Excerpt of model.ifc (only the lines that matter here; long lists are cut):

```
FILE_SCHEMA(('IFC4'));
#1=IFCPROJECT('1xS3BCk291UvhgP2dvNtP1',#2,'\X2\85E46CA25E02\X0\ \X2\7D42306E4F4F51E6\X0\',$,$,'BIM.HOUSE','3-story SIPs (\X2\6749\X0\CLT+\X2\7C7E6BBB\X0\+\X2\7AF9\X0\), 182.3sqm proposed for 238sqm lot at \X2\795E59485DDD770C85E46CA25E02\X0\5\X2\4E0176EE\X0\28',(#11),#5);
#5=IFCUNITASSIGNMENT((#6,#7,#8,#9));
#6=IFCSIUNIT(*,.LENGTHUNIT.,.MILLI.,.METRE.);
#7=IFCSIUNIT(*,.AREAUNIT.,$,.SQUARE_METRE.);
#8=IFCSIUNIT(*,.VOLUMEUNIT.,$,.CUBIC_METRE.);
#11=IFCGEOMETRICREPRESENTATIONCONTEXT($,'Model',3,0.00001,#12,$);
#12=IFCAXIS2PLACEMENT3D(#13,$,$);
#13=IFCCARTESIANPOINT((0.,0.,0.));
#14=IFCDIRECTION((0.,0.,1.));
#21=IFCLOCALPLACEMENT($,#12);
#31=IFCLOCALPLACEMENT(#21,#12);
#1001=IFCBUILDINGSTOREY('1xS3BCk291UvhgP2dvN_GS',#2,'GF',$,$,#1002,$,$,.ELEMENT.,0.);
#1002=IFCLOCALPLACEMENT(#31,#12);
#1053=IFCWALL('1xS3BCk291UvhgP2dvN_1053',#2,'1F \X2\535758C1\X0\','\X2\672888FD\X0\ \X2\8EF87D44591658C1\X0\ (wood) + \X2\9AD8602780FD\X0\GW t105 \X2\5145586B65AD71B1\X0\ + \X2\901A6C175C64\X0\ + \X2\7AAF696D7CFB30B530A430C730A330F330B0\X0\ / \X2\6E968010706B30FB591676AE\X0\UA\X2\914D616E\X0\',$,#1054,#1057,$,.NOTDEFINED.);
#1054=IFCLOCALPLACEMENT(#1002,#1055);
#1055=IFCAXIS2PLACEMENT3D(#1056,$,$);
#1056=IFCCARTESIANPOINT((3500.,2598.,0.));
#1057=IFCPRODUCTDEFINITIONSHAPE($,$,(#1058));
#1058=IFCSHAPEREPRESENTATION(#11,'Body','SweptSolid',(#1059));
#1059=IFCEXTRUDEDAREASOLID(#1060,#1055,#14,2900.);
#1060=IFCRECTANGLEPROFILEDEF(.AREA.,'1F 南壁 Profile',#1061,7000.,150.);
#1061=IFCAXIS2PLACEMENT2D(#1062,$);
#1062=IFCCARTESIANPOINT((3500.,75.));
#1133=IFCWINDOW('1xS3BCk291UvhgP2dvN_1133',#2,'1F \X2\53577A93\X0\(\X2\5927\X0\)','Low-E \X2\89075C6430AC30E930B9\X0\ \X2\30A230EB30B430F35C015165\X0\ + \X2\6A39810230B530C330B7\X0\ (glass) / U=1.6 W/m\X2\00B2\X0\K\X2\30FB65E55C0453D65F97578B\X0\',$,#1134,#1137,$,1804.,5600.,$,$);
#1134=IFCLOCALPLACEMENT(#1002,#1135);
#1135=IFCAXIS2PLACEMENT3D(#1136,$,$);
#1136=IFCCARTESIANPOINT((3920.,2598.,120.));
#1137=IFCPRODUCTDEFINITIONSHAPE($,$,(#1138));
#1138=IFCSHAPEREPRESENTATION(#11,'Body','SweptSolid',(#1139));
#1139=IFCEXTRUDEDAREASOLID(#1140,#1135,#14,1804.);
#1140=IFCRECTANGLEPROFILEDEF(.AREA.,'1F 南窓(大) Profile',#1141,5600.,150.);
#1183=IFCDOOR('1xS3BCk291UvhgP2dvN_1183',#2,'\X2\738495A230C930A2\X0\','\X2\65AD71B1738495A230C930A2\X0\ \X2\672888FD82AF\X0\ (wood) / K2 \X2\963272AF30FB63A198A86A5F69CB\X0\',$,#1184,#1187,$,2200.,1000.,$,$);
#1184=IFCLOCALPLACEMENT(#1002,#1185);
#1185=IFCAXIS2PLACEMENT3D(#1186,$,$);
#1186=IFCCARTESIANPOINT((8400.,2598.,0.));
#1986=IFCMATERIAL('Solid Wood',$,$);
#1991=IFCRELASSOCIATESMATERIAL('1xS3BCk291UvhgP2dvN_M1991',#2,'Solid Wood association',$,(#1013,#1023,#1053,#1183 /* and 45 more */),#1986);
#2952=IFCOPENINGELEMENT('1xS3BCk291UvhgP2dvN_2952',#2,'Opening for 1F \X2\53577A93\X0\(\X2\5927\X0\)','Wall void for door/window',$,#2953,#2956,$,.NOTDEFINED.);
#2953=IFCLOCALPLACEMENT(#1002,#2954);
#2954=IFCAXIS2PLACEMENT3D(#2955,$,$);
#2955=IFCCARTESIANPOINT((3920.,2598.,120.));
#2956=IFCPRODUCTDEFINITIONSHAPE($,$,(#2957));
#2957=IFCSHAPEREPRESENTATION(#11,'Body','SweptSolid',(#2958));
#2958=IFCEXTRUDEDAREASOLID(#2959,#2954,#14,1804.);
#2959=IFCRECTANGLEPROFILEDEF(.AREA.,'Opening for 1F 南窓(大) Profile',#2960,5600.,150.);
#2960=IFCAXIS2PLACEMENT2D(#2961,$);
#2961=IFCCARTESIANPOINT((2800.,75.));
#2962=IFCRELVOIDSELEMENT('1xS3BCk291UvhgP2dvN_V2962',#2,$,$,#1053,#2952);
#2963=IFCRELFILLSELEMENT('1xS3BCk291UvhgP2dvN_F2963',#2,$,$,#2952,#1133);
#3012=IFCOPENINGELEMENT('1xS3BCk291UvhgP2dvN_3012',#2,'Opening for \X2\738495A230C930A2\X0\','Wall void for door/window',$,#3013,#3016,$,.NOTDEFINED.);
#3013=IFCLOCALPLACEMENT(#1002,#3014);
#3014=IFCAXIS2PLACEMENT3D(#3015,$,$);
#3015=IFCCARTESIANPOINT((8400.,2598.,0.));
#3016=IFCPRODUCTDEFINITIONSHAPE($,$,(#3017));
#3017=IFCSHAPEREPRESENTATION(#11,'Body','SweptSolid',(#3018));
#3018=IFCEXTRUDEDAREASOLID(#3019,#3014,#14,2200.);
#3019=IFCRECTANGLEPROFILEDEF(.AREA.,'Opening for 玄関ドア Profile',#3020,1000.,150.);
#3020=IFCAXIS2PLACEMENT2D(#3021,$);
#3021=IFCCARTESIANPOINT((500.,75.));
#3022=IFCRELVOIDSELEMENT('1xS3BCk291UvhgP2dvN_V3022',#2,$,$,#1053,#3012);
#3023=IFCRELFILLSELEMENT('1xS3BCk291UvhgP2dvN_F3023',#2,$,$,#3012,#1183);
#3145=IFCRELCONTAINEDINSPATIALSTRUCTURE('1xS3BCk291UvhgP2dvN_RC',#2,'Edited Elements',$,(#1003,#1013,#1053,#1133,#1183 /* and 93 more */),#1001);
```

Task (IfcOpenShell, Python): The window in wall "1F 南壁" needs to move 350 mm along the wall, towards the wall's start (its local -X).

```python
import ifcopenshell
import ifcopenshell.api.geometry
import ifcopenshell.util.placement

model = ifcopenshell.open("model.ifc")

window = model.by_id(1133)
opening = window.FillsVoids[0].RelatingOpeningElement
wall = opening.VoidsElements[0].RelatingBuildingElement

wall_matrix = ifcopenshell.util.placement.get_local_placement(wall.ObjectPlacement)
shift = wall_matrix[:3, 0] * -350.0
before = ifcopenshell.util.placement.get_local_placement(window.ObjectPlacement)[:3, 3].copy()

# The window is not placed relative to its opening, so move both.
for product in (opening, window):
    matrix = ifcopenshell.util.placement.get_local_placement(product.ObjectPlacement)
    matrix[:3, 3] += shift
    ifcopenshell.api.geometry.edit_object_placement(model, product=product, matrix=matrix, is_si=False)

after = ifcopenshell.util.placement.get_local_placement(window.ObjectPlacement)[:3, 3]
print("window moved by", (after - before).round(3) + 0.0)

model.write("model_rev.ifc")
```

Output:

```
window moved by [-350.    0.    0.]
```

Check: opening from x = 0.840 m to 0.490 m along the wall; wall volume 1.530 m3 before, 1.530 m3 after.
